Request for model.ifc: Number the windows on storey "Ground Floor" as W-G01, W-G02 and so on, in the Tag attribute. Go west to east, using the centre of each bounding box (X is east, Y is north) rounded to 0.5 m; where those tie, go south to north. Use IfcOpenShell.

First a look at what the model holds.

```python
import ifcopenshell
import ifcopenshell.util.element
import ifcopenshell.util.placement

model = ifcopenshell.open("model.ifc")
print(model.schema)
storey = next(s for s in model.by_type("IfcBuildingStorey") if s.Name == "Ground Floor")
windows = [e for e in ifcopenshell.util.element.get_decomposition(storey) if e.is_a("IfcWindow")]
for e in sorted(windows, key=lambda e: e.id()):
    origin = ifcopenshell.util.placement.get_local_placement(e.ObjectPlacement)[:3, 3]
    print(e.id(), e.Tag, e.Name, origin.round(2) + 0.0, sep=" | ")
```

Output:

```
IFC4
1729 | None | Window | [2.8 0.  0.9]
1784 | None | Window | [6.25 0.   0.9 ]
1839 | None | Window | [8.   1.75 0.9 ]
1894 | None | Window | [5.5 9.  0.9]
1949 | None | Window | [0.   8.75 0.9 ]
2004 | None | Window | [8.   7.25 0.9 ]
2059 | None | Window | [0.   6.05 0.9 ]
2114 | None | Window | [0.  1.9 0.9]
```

```python
import ifcopenshell
import ifcopenshell.geom
import ifcopenshell.util.element
import ifcopenshell.util.shape

model = ifcopenshell.open("model.ifc")
settings = ifcopenshell.geom.settings()
settings.set("use-world-coords", True)


def centre(element):
    shape = ifcopenshell.geom.create_shape(settings, element)
    return ifcopenshell.util.shape.get_bbox_centroid(shape.geometry)


storey = next(s for s in model.by_type("IfcBuildingStorey") if s.Name == "Ground Floor")
windows = [e for e in ifcopenshell.util.element.get_decomposition(storey) if e.is_a("IfcWindow")]

# Insertion points can sit at a corner or the storey origin, so sort by the geometry (in metres).
centres = {e: centre(e) for e in windows}
windows.sort(key=lambda e: (round(centres[e][0] / 0.5), centres[e][1]))

for i, e in enumerate(windows, start=1):
    number = f"W-G{i:02d}"
    e.Tag = number
    print(e.id(), number)

model.write("model-out.ifc")
```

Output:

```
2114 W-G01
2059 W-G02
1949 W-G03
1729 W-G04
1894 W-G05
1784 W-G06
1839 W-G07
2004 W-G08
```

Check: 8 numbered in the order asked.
